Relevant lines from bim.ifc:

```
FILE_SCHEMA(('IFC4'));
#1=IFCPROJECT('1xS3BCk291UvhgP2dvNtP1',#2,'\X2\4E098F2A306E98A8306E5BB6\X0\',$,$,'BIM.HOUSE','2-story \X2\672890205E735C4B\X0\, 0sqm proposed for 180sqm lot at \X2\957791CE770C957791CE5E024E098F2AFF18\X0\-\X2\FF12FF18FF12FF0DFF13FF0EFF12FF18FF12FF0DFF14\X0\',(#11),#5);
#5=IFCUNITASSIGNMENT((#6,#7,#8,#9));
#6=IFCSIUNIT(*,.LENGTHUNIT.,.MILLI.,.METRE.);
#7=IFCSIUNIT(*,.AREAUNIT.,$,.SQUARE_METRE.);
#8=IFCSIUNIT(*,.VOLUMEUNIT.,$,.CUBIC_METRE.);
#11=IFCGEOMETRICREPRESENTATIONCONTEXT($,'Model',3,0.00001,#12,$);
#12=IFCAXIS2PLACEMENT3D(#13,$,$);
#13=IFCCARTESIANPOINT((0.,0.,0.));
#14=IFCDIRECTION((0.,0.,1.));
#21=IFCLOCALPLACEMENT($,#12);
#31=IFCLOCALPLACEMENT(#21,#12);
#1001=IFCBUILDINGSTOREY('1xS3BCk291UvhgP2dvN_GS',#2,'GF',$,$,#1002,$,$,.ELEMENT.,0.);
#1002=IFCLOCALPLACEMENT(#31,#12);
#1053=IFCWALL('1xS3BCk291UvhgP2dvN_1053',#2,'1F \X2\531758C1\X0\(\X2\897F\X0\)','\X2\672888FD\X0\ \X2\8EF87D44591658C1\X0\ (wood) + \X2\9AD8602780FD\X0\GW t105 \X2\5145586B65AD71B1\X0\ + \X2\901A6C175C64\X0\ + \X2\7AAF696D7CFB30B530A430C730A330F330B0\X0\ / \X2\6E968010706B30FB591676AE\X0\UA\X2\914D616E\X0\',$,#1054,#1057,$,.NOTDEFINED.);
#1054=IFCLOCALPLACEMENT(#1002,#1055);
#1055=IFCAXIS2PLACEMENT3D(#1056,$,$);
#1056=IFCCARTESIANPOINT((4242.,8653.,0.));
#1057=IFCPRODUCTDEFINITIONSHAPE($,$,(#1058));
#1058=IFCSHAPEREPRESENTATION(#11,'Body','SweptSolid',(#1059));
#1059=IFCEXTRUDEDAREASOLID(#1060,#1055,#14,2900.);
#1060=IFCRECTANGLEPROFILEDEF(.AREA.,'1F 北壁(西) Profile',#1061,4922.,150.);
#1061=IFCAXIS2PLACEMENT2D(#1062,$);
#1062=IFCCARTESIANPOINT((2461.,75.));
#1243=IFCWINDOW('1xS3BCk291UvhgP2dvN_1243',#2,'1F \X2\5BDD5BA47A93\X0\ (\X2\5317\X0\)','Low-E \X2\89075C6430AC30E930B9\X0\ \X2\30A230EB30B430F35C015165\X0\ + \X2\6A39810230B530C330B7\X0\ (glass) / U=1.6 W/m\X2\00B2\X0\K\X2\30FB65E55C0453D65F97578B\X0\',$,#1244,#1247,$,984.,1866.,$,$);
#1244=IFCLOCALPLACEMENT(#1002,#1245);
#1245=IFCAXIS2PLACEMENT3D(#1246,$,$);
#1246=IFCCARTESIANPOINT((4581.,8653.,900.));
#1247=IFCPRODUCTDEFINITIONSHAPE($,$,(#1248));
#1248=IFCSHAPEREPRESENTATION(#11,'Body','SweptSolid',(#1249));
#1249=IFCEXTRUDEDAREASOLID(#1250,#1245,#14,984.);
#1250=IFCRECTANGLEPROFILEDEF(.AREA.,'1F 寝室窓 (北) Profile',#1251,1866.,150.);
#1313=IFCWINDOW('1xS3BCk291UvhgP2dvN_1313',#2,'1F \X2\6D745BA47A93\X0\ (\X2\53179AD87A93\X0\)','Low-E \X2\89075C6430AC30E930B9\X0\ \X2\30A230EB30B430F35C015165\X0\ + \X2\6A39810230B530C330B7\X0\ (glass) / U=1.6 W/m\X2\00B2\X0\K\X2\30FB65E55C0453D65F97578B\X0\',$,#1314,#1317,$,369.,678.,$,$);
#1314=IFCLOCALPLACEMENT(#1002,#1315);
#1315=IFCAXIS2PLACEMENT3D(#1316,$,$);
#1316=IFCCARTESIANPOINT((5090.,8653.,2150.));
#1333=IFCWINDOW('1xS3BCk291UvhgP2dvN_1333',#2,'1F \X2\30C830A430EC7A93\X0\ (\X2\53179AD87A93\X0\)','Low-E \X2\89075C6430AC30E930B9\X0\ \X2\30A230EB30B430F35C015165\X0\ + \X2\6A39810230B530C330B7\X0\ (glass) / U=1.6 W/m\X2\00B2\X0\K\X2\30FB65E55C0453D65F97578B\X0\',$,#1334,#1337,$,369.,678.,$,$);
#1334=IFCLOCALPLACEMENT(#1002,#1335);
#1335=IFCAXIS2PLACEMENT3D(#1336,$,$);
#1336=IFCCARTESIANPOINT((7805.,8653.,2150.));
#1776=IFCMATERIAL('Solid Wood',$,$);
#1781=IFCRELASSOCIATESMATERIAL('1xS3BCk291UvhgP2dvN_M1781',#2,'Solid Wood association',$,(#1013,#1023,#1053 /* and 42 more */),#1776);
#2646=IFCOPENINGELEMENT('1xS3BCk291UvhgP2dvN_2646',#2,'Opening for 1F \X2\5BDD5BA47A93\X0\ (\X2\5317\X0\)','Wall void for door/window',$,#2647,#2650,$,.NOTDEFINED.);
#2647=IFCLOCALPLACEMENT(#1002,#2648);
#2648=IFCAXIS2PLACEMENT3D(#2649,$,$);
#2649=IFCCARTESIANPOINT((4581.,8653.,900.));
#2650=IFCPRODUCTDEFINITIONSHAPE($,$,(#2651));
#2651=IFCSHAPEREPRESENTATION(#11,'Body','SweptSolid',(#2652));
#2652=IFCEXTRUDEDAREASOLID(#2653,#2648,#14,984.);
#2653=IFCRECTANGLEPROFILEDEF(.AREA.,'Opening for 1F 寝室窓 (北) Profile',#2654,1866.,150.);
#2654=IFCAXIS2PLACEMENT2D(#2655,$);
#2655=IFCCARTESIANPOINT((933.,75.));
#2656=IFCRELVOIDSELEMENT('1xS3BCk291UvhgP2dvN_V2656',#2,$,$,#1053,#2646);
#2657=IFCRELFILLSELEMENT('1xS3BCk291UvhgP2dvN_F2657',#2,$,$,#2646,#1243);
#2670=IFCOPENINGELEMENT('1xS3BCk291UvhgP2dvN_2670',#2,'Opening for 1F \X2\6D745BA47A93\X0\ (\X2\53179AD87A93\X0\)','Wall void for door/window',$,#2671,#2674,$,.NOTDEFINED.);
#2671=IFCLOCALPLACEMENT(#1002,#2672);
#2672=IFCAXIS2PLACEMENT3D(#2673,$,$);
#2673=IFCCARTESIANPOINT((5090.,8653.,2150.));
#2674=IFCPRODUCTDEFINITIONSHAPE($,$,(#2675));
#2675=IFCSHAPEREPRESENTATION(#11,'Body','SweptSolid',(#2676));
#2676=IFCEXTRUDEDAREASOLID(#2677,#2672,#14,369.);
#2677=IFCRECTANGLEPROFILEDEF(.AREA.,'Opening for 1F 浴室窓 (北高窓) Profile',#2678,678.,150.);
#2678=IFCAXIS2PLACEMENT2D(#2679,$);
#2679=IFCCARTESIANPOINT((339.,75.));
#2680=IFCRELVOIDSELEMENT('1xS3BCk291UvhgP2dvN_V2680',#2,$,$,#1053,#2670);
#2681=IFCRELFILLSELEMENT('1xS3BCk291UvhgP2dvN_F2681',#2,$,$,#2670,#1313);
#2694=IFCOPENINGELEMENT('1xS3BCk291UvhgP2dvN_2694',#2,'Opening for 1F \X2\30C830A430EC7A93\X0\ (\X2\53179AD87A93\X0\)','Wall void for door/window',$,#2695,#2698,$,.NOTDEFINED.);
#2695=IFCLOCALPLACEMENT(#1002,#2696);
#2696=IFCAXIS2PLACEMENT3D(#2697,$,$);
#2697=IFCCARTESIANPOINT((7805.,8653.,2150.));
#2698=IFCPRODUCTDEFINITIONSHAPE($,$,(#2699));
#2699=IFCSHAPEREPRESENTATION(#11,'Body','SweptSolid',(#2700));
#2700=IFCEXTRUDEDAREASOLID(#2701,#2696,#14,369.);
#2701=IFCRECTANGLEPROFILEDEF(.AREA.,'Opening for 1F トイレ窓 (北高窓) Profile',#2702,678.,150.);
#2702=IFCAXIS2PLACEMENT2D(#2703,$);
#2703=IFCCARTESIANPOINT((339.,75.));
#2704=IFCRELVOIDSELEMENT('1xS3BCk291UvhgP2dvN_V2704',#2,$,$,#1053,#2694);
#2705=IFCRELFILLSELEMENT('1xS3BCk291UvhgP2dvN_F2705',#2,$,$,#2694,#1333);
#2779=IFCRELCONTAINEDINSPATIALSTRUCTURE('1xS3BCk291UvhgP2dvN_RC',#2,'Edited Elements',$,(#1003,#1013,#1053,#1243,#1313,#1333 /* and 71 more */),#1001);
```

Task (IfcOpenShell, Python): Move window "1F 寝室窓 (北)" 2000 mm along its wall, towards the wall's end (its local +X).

```python
import ifcopenshell
import ifcopenshell.api.geometry
import ifcopenshell.util.placement
import ifcopenshell.util.unit

model = ifcopenshell.open("bim.ifc")
unit_scale = ifcopenshell.util.unit.calculate_unit_scale(model)

window = model.by_guid("1xS3BCk291UvhgP2dvN_1243")
opening = window.FillsVoids[0].RelatingOpeningElement
wall = opening.VoidsElements[0].RelatingBuildingElement

wall_matrix = ifcopenshell.util.placement.get_local_placement(wall.ObjectPlacement)
shift = wall_matrix[:3, 0] * 2 / unit_scale
before = ifcopenshell.util.placement.get_local_placement(window.ObjectPlacement)[:3, 3].copy()

# The window is not placed relative to its opening, so move both.
for product in (opening, window):
    matrix = ifcopenshell.util.placement.get_local_placement(product.ObjectPlacement)
    matrix[:3, 3] += shift
    ifcopenshell.api.geometry.edit_object_placement(model, product=product, matrix=matrix, is_si=False)

after = ifcopenshell.util.placement.get_local_placement(window.ObjectPlacement)[:3, 3]
print("window moved by", (after - before).round(3) + 0.0)

model.write("bim_edited.ifc")
```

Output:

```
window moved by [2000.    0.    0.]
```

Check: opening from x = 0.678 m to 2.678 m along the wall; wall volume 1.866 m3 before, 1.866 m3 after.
